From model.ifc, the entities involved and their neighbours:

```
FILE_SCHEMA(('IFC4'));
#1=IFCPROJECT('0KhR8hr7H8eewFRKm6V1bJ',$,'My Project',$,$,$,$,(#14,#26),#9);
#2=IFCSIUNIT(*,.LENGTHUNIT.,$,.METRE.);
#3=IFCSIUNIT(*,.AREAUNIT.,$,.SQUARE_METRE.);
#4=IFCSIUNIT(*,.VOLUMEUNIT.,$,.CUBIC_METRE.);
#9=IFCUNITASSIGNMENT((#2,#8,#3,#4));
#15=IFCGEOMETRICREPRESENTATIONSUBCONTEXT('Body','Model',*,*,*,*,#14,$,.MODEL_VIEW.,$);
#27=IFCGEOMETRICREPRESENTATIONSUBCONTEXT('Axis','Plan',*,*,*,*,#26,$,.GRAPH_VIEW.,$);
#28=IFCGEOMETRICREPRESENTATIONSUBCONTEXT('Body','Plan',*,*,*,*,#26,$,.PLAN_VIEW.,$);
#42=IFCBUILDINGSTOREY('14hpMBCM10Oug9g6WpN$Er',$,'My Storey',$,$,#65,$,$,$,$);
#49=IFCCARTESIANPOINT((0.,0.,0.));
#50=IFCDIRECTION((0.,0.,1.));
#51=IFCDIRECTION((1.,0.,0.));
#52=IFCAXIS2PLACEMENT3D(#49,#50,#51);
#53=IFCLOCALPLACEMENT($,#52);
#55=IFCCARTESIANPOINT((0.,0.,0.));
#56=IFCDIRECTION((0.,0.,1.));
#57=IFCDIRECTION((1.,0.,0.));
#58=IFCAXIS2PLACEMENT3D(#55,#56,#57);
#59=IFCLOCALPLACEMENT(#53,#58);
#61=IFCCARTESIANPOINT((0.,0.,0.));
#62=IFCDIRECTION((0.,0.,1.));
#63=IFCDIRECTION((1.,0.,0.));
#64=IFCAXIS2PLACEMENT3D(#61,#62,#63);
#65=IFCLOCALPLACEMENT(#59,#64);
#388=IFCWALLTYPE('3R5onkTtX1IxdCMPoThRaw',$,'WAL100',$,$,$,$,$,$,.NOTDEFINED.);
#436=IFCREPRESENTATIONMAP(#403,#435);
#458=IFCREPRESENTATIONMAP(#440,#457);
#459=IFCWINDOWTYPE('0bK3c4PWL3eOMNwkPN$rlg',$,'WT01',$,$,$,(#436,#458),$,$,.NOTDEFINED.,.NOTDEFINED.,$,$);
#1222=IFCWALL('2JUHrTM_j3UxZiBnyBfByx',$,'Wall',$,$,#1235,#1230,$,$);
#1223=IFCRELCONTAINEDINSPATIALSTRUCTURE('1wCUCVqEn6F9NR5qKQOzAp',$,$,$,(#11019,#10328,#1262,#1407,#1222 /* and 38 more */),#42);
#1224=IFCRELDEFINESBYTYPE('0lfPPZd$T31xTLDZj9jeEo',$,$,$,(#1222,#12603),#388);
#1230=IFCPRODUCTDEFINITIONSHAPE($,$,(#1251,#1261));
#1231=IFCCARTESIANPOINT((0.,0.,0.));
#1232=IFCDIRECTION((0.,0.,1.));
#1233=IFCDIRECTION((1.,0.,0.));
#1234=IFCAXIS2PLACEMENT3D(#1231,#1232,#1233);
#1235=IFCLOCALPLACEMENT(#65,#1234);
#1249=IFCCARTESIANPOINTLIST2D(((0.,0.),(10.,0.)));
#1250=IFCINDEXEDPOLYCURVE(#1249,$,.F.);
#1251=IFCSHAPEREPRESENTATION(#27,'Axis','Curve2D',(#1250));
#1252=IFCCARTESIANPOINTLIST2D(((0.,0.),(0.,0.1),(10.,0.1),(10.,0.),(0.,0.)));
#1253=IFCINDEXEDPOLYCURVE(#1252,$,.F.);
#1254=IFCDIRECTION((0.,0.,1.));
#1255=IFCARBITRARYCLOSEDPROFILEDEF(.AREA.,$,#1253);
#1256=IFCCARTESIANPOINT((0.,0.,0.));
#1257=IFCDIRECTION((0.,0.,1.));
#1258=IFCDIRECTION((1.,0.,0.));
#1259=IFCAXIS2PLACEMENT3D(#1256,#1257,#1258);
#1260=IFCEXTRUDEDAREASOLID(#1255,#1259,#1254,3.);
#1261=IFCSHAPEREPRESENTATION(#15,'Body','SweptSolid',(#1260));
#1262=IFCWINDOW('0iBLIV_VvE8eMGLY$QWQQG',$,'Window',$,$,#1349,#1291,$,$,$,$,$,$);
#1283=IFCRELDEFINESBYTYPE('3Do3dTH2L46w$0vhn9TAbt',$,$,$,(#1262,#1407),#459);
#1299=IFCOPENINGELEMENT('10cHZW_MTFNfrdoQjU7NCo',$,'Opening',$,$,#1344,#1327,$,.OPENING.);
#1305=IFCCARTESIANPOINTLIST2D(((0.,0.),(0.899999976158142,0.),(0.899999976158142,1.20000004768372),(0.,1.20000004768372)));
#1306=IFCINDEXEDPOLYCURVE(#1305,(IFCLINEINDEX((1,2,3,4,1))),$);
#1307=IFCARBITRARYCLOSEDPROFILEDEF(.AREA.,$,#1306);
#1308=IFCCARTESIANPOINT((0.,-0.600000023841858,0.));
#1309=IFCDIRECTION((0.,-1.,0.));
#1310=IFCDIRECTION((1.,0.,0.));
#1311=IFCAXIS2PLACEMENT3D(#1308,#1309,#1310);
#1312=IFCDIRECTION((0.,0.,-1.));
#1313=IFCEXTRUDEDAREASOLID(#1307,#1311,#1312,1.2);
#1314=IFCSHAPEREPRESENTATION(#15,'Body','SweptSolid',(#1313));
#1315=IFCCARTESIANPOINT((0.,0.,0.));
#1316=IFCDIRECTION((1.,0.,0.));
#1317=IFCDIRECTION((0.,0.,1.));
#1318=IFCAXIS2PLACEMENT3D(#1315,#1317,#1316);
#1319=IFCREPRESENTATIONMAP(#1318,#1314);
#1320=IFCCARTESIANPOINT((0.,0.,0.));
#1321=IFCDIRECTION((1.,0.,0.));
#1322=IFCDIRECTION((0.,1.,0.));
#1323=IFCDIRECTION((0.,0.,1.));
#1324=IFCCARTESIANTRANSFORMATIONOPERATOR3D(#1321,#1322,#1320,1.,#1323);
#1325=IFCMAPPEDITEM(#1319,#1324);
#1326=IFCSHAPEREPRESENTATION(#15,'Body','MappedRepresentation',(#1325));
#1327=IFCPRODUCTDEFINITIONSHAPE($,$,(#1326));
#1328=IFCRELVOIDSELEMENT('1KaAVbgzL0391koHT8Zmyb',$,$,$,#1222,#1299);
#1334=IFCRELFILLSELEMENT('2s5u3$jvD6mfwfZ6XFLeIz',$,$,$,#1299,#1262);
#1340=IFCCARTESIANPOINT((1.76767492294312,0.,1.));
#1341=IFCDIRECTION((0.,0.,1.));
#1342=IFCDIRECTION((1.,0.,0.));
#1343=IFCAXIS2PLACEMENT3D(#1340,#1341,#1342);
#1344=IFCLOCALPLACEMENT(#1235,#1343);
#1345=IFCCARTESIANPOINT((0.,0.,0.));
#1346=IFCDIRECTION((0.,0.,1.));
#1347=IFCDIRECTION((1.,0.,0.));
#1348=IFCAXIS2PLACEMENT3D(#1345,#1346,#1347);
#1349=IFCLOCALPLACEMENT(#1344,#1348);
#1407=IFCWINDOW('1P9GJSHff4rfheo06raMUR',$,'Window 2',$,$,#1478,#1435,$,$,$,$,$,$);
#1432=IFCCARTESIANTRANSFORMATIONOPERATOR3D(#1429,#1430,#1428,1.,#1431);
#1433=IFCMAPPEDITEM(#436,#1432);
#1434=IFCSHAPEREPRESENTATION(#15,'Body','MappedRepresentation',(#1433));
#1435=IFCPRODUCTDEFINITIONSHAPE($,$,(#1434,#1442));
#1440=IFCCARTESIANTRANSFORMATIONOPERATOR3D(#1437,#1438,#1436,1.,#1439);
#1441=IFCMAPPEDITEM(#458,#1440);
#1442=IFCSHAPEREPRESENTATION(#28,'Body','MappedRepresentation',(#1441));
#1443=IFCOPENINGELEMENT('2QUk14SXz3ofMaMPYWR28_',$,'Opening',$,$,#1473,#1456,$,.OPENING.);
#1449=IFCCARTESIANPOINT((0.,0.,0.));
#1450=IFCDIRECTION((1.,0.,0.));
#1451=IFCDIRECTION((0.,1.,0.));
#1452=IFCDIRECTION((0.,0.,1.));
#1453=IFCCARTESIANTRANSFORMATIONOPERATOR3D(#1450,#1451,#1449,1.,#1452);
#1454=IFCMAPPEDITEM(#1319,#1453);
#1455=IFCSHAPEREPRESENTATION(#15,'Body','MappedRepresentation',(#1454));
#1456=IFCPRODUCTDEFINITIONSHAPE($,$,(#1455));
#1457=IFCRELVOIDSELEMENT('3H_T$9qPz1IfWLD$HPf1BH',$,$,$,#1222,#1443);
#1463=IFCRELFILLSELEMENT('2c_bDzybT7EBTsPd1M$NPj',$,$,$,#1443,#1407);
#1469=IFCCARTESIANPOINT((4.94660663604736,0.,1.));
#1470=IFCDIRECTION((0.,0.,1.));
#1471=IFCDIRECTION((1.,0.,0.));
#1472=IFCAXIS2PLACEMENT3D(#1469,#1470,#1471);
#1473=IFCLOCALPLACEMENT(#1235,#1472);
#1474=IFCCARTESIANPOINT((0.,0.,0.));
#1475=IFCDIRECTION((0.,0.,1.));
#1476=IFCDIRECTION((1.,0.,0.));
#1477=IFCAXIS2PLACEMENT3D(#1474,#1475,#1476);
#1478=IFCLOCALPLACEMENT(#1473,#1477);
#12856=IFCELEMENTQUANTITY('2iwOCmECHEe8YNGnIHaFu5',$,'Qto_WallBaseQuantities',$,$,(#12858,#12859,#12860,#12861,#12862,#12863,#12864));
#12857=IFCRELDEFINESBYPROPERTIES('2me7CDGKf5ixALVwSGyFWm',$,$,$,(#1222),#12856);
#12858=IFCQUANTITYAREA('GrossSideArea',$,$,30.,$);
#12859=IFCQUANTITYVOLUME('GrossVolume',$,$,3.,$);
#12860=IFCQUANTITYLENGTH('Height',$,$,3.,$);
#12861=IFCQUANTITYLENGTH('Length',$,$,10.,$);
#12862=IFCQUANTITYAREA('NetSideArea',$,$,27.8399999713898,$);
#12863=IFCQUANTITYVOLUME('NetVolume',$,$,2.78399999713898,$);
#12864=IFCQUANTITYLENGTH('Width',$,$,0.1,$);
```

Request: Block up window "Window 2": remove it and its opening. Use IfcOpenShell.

```python
import ifcopenshell
import ifcopenshell.api.feature
import ifcopenshell.api.pset
import ifcopenshell.api.root
import ifcopenshell.geom
import ifcopenshell.util.element
import ifcopenshell.util.shape
import ifcopenshell.util.unit

model = ifcopenshell.open("model.ifc")
area_scale = ifcopenshell.util.unit.calculate_unit_scale(model, "AREAUNIT")
volume_scale = ifcopenshell.util.unit.calculate_unit_scale(model, "VOLUMEUNIT")
settings = ifcopenshell.geom.settings()


def volume(element):
    """Net volume in cubic metres, openings subtracted."""
    shape = ifcopenshell.geom.create_shape(settings, element)
    return ifcopenshell.util.shape.get_volume(shape.geometry)


window = model.by_guid("1P9GJSHff4rfheo06raMUR")
opening = window.FillsVoids[0].RelatingOpeningElement
wall = opening.VoidsElements[0].RelatingBuildingElement
before = volume(wall)

ifcopenshell.api.root.remove_product(model, product=window)
ifcopenshell.api.feature.remove_feature(model, feature=opening)

after = volume(wall)
thickness = 0.1  # wall thickness in metres

# Update the wall's stored quantities.
qto = model.by_id(ifcopenshell.util.element.get_pset(wall, "Qto_WallBaseQuantities", should_inherit=False)["id"])
ifcopenshell.api.pset.edit_qto(model, qto=qto, properties={
    "NetSideArea": after / thickness / area_scale,
    "NetVolume": after / volume_scale,
})

print(f"wall volume {before:.3f} -> {after:.3f} m3")

model.write("model_rev.ifc")
```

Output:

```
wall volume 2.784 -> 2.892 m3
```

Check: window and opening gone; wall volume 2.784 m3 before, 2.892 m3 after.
